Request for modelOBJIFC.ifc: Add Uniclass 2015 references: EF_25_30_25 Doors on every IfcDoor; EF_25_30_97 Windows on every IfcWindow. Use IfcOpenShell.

First a look at what the model holds.

```python
import ifcopenshell

model = ifcopenshell.open("modelOBJIFC.ifc")
print(model.schema)
print("classifications:", [c.Name for c in model.by_type("IfcClassification")])
for ifc_class in ("IfcDoor", "IfcRoof", "IfcStair", "IfcWall", "IfcWindow"):
    print(ifc_class, len(model.by_type(ifc_class)))
```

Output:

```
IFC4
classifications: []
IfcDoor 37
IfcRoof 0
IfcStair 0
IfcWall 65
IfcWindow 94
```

```python
import ifcopenshell
import ifcopenshell.api.classification

model = ifcopenshell.open("modelOBJIFC.ifc")

system = ifcopenshell.api.classification.add_classification(model, classification="Uniclass 2015")

codes = {
    "IfcDoor": ("EF_25_30_25", "Doors"),
    "IfcWindow": ("EF_25_30_97", "Windows"),
}
for ifc_class, (code, name) in codes.items():
    products = model.by_type(ifc_class)
    ifcopenshell.api.classification.add_reference(
        model, products=products, classification=system, identification=code, name=name
    )
    print(code, len(products))

model.write("modelOBJIFC_updated.ifc")
```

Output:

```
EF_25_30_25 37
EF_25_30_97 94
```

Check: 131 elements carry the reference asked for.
